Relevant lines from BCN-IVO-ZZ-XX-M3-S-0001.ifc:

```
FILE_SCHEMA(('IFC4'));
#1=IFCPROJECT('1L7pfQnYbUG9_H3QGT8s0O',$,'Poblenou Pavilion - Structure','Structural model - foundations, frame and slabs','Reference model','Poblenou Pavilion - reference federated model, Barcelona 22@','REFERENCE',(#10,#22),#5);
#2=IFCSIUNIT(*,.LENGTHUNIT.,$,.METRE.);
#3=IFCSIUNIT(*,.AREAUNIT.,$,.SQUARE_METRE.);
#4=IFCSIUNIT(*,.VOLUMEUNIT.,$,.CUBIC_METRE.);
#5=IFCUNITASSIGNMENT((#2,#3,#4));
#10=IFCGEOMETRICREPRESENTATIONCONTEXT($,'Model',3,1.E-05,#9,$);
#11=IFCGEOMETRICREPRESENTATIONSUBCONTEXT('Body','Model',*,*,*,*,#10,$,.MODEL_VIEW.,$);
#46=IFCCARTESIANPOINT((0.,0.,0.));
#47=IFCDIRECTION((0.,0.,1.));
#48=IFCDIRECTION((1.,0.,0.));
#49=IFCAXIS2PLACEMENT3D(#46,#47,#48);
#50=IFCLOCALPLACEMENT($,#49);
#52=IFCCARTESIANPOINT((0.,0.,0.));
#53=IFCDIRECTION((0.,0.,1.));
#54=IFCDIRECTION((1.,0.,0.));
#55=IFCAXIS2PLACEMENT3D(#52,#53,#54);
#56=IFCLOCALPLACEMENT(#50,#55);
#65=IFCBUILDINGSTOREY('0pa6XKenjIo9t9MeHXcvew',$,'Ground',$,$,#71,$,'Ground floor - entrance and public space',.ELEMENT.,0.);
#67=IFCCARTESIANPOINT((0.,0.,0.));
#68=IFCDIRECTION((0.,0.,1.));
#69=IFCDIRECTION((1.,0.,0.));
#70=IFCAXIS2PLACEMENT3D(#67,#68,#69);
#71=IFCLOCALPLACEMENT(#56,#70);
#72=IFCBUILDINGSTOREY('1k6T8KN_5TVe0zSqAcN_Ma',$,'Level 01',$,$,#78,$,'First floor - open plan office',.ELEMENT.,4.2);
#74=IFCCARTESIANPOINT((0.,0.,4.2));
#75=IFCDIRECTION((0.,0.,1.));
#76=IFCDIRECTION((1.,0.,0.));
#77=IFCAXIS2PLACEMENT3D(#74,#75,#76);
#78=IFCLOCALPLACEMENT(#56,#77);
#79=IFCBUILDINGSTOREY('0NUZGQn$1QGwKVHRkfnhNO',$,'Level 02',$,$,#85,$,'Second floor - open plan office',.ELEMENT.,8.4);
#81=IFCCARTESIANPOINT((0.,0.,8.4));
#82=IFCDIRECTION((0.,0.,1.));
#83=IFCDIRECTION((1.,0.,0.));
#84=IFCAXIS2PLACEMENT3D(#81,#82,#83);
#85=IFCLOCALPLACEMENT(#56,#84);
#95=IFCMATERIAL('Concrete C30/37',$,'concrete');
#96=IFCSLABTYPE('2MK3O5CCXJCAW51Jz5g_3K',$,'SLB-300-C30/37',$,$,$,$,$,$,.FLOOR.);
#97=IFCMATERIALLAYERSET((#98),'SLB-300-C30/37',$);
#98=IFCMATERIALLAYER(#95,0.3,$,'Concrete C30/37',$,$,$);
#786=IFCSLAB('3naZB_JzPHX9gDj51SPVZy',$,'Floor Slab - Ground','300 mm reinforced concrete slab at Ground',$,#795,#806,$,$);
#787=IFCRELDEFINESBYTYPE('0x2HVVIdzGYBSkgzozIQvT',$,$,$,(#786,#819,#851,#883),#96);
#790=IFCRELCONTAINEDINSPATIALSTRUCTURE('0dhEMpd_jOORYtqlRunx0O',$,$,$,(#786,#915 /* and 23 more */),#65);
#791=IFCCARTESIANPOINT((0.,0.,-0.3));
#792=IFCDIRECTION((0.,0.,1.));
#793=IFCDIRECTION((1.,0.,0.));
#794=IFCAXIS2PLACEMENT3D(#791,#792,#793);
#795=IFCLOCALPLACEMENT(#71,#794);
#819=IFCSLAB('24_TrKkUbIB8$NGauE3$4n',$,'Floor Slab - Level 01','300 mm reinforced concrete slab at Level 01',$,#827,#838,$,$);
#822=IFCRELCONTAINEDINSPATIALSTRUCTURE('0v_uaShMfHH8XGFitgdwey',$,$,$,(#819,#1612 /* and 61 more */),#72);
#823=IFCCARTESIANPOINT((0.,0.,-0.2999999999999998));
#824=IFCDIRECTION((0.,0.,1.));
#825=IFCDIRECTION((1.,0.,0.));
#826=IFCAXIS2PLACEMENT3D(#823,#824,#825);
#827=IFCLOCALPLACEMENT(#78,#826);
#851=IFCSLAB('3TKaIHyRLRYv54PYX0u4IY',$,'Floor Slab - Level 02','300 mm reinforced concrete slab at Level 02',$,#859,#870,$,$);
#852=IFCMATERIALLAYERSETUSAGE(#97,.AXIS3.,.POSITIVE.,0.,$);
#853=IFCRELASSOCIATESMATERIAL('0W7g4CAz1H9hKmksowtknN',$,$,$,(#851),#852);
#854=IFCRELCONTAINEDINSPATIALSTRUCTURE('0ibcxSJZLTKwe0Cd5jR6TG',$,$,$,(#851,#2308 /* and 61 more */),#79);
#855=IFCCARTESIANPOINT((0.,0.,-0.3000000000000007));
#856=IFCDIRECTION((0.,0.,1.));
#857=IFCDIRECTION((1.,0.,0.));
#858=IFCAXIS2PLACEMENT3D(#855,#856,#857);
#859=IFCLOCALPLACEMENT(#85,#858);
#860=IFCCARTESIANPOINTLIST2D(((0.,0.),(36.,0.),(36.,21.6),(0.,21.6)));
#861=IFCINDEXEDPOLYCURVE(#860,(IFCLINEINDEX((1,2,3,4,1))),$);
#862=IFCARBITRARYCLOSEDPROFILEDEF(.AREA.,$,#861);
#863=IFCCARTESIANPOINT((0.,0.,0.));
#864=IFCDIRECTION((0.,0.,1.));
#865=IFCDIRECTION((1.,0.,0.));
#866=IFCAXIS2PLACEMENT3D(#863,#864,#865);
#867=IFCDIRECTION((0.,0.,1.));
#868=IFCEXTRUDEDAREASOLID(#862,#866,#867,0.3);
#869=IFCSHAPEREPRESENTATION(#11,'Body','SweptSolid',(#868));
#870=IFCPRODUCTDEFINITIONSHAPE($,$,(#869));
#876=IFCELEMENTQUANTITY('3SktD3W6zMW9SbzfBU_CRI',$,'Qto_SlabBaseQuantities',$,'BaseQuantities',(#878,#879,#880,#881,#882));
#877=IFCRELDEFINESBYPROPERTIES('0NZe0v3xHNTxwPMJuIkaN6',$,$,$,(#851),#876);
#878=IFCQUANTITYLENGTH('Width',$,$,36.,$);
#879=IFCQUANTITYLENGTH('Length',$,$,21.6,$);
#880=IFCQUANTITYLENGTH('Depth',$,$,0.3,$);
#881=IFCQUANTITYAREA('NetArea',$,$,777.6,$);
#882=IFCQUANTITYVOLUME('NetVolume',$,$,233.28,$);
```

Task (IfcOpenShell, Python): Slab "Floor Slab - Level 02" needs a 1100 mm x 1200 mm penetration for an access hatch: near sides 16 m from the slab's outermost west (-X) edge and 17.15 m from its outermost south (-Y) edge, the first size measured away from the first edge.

```python
import numpy as np
import ifcopenshell
import ifcopenshell.api.feature
import ifcopenshell.api.geometry
import ifcopenshell.api.pset
import ifcopenshell.api.root
import ifcopenshell.geom
import ifcopenshell.util.element
import ifcopenshell.util.placement
import ifcopenshell.util.representation
import ifcopenshell.util.shape
import ifcopenshell.util.unit

model = ifcopenshell.open("BCN-IVO-ZZ-XX-M3-S-0001.ifc")
unit_scale = ifcopenshell.util.unit.calculate_unit_scale(model)
area_scale = ifcopenshell.util.unit.calculate_unit_scale(model, "AREAUNIT")
volume_scale = ifcopenshell.util.unit.calculate_unit_scale(model, "VOLUMEUNIT")
settings = ifcopenshell.geom.settings()


def volume(element):
    """Net volume in cubic metres, openings subtracted."""
    shape = ifcopenshell.geom.create_shape(settings, element)
    return ifcopenshell.util.shape.get_volume(shape.geometry)


slab = model.by_guid("3TKaIHyRLRYv54PYX0u4IY")
before = volume(slab)

# Extent in the slab's own axes, in metres. The edges named are its -X and -Y sides.
slab_shape = ifcopenshell.geom.create_shape(settings, slab)
vertices = ifcopenshell.util.shape.get_vertices(slab_shape.geometry)
x_min, y_min, bottom = vertices.min(axis=0)
top = vertices[:, 2].max()

opening = ifcopenshell.api.root.create_entity(model, ifc_class="IfcOpeningElement", name="Access hatch opening", predefined_type="OPENING")
context = ifcopenshell.util.representation.get_context(model, "Model", "Body", "MODEL_VIEW")
width, depth = 1.1, 1.2
outline = [(0.0, 0.0), (width, 0.0), (width, depth), (0.0, depth), (0.0, 0.0)]
# Overshoot both faces by 50 mm so the cut is clean.
shape = ifcopenshell.api.geometry.add_slab_representation(
    model, context=context, depth=top - bottom + 0.1, polyline=outline
)
ifcopenshell.api.geometry.assign_representation(model, product=opening, representation=shape)

matrix = ifcopenshell.util.placement.get_local_placement(slab.ObjectPlacement)
matrix[:, 3] = matrix @ np.append(np.array([x_min + 16, y_min + 17.15, bottom - 0.05]) / unit_scale, 1.0)
ifcopenshell.api.geometry.edit_object_placement(model, product=opening, matrix=matrix, is_si=False)
ifcopenshell.api.feature.add_feature(model, feature=opening, element=slab)

after = volume(slab)

# Update the slab's stored quantities.
qto = model.by_id(ifcopenshell.util.element.get_pset(slab, "Qto_SlabBaseQuantities", should_inherit=False)["id"])
ifcopenshell.api.pset.edit_qto(model, qto=qto, properties={
    "NetArea": after / (top - bottom) / area_scale,
    "NetVolume": after / volume_scale,
})

print(f"slab volume {before:.3f} -> {after:.3f} m3")

model.write("BCN-IVO-ZZ-XX-M3-S-0001-out.ifc")
```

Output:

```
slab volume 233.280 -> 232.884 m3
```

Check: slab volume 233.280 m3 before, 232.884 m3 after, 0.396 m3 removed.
